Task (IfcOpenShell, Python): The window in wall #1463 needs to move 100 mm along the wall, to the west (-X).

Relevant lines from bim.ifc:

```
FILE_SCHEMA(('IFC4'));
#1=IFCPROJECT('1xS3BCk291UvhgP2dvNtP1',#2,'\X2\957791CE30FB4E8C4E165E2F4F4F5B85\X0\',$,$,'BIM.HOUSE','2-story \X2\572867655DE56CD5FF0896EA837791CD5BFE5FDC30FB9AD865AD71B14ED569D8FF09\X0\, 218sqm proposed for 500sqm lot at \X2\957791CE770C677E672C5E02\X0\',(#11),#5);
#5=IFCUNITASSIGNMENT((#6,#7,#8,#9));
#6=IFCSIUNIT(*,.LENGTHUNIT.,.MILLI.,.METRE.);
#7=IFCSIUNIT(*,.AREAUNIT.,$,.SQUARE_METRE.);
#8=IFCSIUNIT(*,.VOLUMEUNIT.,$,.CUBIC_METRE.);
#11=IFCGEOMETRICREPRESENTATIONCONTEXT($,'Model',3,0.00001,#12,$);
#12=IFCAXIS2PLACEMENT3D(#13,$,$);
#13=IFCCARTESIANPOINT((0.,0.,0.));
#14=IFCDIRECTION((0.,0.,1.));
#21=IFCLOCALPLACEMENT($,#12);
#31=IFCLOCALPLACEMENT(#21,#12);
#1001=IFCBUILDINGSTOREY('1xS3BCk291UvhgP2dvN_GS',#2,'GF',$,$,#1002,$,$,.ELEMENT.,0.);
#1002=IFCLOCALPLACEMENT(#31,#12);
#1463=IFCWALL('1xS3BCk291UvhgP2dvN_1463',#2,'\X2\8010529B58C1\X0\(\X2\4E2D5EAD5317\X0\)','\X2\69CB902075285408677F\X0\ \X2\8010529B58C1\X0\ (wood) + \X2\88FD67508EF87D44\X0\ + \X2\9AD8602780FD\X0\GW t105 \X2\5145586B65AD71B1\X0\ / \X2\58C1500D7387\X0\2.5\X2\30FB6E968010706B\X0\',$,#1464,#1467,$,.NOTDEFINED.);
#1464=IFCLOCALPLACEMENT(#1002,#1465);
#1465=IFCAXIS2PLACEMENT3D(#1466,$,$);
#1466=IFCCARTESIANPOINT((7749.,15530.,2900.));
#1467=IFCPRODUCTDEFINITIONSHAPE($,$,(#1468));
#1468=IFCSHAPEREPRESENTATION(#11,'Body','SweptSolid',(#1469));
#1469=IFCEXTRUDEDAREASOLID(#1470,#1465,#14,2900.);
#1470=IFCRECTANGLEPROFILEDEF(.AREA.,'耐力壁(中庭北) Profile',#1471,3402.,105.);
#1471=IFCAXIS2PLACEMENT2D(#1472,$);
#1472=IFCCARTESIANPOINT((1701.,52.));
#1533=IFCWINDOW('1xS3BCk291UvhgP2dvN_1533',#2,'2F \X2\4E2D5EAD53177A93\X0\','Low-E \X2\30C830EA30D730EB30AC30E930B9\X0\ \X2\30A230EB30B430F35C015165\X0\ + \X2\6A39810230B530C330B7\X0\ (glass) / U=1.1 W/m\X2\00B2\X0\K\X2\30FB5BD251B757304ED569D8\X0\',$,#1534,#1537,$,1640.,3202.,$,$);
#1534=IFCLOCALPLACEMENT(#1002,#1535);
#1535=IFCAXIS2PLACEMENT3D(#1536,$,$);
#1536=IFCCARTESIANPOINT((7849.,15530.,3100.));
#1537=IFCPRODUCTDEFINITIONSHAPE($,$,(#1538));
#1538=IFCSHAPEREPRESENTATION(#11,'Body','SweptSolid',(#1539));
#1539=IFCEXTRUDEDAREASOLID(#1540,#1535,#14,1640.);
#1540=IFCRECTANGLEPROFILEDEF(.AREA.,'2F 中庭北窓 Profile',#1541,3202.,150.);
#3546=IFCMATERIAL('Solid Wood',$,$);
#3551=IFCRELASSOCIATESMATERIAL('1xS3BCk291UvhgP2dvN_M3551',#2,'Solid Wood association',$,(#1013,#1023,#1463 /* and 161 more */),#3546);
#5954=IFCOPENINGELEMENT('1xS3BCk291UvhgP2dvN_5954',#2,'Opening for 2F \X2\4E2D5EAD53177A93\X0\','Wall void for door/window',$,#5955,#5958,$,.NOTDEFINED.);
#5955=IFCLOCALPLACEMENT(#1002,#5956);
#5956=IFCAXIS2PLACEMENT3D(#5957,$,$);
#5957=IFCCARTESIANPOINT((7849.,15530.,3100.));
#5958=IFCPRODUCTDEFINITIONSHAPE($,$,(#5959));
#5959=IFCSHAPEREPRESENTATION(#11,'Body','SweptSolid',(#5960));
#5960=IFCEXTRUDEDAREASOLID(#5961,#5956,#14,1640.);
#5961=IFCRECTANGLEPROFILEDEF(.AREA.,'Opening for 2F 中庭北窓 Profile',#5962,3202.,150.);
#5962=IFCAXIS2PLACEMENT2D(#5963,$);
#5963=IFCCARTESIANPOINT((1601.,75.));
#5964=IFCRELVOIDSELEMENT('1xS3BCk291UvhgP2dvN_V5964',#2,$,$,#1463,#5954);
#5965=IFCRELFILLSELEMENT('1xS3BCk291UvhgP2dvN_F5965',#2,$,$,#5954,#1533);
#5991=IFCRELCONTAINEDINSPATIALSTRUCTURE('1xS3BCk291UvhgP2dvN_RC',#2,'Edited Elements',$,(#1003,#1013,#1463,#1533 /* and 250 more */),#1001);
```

```python
import ifcopenshell
import ifcopenshell.api.geometry
import ifcopenshell.util.placement
import ifcopenshell.util.unit

model = ifcopenshell.open("bim.ifc")
unit_scale = ifcopenshell.util.unit.calculate_unit_scale(model)

window = model.by_guid("1xS3BCk291UvhgP2dvN_1533")
opening = window.FillsVoids[0].RelatingOpeningElement
wall = opening.VoidsElements[0].RelatingBuildingElement

wall_matrix = ifcopenshell.util.placement.get_local_placement(wall.ObjectPlacement)
shift = wall_matrix[:3, 0] * -0.1 / unit_scale
before = ifcopenshell.util.placement.get_local_placement(window.ObjectPlacement)[:3, 3].copy()

# The window is not placed relative to its opening, so move both.
for product in (opening, window):
    matrix = ifcopenshell.util.placement.get_local_placement(product.ObjectPlacement)
    matrix[:3, 3] += shift
    ifcopenshell.api.geometry.edit_object_placement(model, product=product, matrix=matrix, is_si=False)

after = ifcopenshell.util.placement.get_local_placement(window.ObjectPlacement)[:3, 3]
print("window moved by", (after - before).round(3) + 0.0)

model.write("bim_edited.ifc")
```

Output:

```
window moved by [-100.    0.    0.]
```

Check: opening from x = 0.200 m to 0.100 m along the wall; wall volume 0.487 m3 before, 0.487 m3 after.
